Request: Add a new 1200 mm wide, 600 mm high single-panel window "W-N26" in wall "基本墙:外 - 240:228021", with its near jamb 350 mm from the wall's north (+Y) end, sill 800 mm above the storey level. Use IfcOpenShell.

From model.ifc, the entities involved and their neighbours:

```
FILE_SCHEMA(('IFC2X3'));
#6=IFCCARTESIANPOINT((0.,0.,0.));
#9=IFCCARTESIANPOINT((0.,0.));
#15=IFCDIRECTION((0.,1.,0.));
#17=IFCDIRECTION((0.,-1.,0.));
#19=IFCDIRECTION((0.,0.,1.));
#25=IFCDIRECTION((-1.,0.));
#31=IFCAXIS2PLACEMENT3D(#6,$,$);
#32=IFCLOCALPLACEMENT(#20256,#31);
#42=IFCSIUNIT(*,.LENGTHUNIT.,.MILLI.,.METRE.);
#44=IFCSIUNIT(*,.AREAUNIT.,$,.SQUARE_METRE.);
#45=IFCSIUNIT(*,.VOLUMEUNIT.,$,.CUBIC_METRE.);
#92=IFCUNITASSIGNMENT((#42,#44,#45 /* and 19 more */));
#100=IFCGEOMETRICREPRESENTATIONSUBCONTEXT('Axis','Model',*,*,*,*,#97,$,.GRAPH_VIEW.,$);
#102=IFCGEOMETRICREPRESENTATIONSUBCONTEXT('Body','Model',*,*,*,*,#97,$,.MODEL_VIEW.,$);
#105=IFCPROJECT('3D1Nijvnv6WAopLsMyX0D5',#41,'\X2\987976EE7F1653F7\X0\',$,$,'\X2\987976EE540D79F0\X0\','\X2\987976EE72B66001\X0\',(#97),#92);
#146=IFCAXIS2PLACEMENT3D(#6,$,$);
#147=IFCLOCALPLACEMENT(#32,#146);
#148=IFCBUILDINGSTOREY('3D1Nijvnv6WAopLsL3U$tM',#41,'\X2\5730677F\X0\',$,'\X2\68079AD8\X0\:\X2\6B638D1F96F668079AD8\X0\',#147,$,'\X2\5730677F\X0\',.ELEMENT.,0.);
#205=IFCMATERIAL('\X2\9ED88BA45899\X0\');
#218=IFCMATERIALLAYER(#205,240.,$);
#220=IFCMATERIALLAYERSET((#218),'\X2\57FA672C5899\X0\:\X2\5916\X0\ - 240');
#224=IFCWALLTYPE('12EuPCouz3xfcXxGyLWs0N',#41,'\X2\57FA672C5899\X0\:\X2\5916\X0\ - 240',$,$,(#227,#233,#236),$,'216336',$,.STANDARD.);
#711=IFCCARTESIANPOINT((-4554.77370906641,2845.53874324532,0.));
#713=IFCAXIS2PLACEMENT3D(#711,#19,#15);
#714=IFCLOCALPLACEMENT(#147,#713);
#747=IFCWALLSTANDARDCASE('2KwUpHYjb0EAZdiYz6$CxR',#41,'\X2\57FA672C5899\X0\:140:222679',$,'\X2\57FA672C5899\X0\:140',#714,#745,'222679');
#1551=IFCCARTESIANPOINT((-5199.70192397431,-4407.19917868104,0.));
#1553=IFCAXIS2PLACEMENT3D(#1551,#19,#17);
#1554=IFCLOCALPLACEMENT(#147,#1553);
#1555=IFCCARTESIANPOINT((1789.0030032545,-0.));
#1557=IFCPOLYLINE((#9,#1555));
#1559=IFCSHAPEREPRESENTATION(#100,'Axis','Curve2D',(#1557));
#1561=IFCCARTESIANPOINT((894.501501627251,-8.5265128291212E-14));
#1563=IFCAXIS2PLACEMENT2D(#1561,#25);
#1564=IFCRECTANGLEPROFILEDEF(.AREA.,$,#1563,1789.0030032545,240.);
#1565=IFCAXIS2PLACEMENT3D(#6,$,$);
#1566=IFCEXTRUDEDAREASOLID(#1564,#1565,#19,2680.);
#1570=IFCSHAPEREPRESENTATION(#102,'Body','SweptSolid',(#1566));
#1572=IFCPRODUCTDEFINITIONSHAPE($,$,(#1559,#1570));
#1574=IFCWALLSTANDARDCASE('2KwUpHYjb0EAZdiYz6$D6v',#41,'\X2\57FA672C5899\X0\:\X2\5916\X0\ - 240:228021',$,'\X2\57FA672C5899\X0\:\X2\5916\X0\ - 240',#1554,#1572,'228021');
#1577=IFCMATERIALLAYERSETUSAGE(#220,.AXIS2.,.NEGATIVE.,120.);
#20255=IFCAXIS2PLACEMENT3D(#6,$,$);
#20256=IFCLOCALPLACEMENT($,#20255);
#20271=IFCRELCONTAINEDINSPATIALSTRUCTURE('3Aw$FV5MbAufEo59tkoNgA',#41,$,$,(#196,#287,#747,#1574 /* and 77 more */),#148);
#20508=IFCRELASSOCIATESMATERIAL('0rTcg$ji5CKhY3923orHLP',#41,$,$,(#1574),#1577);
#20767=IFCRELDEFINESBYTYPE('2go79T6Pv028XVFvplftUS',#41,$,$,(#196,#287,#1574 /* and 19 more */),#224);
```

```python
import numpy as np
import ifcopenshell
import ifcopenshell.api.feature
import ifcopenshell.api.geometry
import ifcopenshell.api.root
import ifcopenshell.api.spatial
import ifcopenshell.api.type
import ifcopenshell.geom
import ifcopenshell.util.element
import ifcopenshell.util.placement
import ifcopenshell.util.representation
import ifcopenshell.util.shape
import ifcopenshell.util.unit

model = ifcopenshell.open("model.ifc")
unit_scale = ifcopenshell.util.unit.calculate_unit_scale(model)
settings = ifcopenshell.geom.settings()


def volume(element):
    """Net volume in cubic metres, openings subtracted."""
    shape = ifcopenshell.geom.create_shape(settings, element)
    return ifcopenshell.util.shape.get_volume(shape.geometry)


wall = model.by_guid("2KwUpHYjb0EAZdiYz6$D6v")
storey = ifcopenshell.util.element.get_container(wall, ifc_class="IfcBuildingStorey")
context = ifcopenshell.util.representation.get_context(model, "Model", "Body", "MODEL_VIEW")
before = volume(wall)

width, height, from_end, sill = 1.2, 0.6, 0.35, 0.8  # metres

# The wall runs along its own X axis, and the end named is its -X end.
wall_shape = ifcopenshell.geom.create_shape(settings, wall)
x, y, z = ifcopenshell.util.shape.get_vertices(wall_shape.geometry).T
start = x.min() + from_end
face, thickness = float(y.min()), float(y.max() - y.min())
wall_matrix = ifcopenshell.util.placement.get_local_placement(wall.ObjectPlacement)
level = ifcopenshell.util.placement.get_local_placement(storey.ObjectPlacement)[2, 3]


def in_wall(x, y):
    """Placement at x, y metres in the wall's axes, at sill height."""
    matrix = wall_matrix.copy()
    matrix[:, 3] = wall_matrix @ np.array([x / unit_scale, y / unit_scale, 0.0, 1.0])
    matrix[2, 3] = level + sill / unit_scale
    return matrix


# Opening: a box that overshoots both wall faces by 50 mm.
opening = ifcopenshell.api.root.create_entity(model, ifc_class="IfcOpeningElement")
box = ifcopenshell.api.geometry.add_wall_representation(
    model, context=context, length=width, height=height, thickness=thickness + 0.1
)
ifcopenshell.api.geometry.assign_representation(model, product=opening, representation=box)
ifcopenshell.api.geometry.edit_object_placement(model, product=opening, matrix=in_wall(start, face - 0.05), is_si=False)
ifcopenshell.api.feature.add_feature(model, feature=opening, element=wall)

window = ifcopenshell.api.root.create_entity(model, ifc_class="IfcWindow", name="W-N26")
window.OverallWidth, window.OverallHeight = width / unit_scale, height / unit_scale
body = ifcopenshell.api.geometry.add_window_representation(
    model,
    context=context,
    overall_width=window.OverallWidth,
    overall_height=window.OverallHeight,
    partition_type="SINGLE_PANEL",
)
ifcopenshell.api.geometry.assign_representation(model, product=window, representation=body)
ifcopenshell.api.spatial.assign_container(model, products=[window], relating_structure=storey)
fills = ifcopenshell.api.feature.add_filling(model, opening=opening, element=window)
fills.OwnerHistory = window.OwnerHistory  # required in IFC2X3

# IFC2X3 keeps the operation on the window style.
style = ifcopenshell.api.root.create_entity(model, ifc_class="IfcWindowStyle", name="W-N26")
style.OperationType, style.ConstructionType = "SINGLE_PANEL", "NOTDEFINED"
style.ParameterTakesPrecedence = style.Sizeable = False
ifcopenshell.api.type.assign_type(model, related_objects=[window], relating_type=style)

# Centre the window in the wall's thickness.
ifcopenshell.api.geometry.edit_object_placement(model, product=window, matrix=in_wall(start, face), is_si=False)
window_shape = ifcopenshell.geom.create_shape(settings, window)
depth = ifcopenshell.util.shape.get_vertices(window_shape.geometry)[:, 1]
offset = face + thickness / 2 - (depth.min() + depth.max()) / 2
ifcopenshell.api.geometry.edit_object_placement(model, product=window, matrix=in_wall(start, offset), is_si=False)

after = volume(wall)

print(f"wall volume {before:.3f} -> {after:.3f} m3")

model.write("model_rev.ifc")
```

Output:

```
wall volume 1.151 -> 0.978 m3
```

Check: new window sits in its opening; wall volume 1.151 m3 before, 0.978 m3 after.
